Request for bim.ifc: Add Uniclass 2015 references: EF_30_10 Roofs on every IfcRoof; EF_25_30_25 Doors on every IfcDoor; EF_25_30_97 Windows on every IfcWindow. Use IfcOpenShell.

First a look at what the model holds.

```python
import ifcopenshell

model = ifcopenshell.open("bim.ifc")
print(model.schema)
print("classifications:", [c.Name for c in model.by_type("IfcClassification")])
for ifc_class in ("IfcDoor", "IfcRoof", "IfcStair", "IfcWall", "IfcWindow"):
    print(ifc_class, len(model.by_type(ifc_class)))
```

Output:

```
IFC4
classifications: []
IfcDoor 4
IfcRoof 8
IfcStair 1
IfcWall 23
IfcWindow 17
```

```python
import ifcopenshell
import ifcopenshell.api.classification

model = ifcopenshell.open("bim.ifc")

system = ifcopenshell.api.classification.add_classification(model, classification="Uniclass 2015")

codes = {
    "IfcRoof": ("EF_30_10", "Roofs"),
    "IfcDoor": ("EF_25_30_25", "Doors"),
    "IfcWindow": ("EF_25_30_97", "Windows"),
}
for ifc_class, (code, name) in codes.items():
    products = model.by_type(ifc_class)
    ifcopenshell.api.classification.add_reference(
        model, products=products, classification=system, identification=code, name=name
    )
    print(code, len(products))

model.write("bim_updated.ifc")
```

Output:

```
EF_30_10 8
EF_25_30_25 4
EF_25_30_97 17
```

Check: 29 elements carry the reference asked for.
